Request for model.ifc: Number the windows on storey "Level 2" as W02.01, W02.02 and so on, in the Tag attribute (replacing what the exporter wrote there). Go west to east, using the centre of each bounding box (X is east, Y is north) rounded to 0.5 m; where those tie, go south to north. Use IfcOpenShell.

First a look at what the model holds.

```python
import ifcopenshell
import ifcopenshell.util.element
import ifcopenshell.util.placement

model = ifcopenshell.open("model.ifc")
print(model.schema)
storey = next(s for s in model.by_type("IfcBuildingStorey") if s.Name == "Level 2")
windows = [e for e in ifcopenshell.util.element.get_decomposition(storey) if e.is_a("IfcWindow")]
for e in sorted(windows, key=lambda e: e.id()):
    origin = ifcopenshell.util.placement.get_local_placement(e.ObjectPlacement)[:3, 3]
    print(e.id(), e.Tag, e.Name, origin.round(2) + 0.0, sep=" | ")
```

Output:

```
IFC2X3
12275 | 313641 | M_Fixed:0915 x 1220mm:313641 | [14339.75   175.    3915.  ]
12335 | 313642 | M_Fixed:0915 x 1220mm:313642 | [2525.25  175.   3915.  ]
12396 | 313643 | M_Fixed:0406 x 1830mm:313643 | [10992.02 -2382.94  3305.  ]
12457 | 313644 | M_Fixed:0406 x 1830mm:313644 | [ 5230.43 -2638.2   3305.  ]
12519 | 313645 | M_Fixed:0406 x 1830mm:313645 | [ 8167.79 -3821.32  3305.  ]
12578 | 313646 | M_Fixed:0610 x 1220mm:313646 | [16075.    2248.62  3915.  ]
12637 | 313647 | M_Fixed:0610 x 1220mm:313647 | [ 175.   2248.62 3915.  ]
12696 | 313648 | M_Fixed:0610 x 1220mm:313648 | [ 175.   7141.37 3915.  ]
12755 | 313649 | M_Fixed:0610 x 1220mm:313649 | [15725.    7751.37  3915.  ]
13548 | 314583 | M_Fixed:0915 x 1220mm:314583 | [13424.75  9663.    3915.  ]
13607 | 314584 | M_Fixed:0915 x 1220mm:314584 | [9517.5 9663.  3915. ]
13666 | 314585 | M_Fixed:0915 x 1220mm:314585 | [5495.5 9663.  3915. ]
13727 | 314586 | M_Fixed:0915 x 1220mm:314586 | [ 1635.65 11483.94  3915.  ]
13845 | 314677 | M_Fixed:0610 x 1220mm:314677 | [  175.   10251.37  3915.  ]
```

```python
import ifcopenshell
import ifcopenshell.geom
import ifcopenshell.util.element
import ifcopenshell.util.shape

model = ifcopenshell.open("model.ifc")
settings = ifcopenshell.geom.settings()
settings.set("use-world-coords", True)


def centre(element):
    shape = ifcopenshell.geom.create_shape(settings, element)
    return ifcopenshell.util.shape.get_bbox_centroid(shape.geometry)


storey = next(s for s in model.by_type("IfcBuildingStorey") if s.Name == "Level 2")
windows = [e for e in ifcopenshell.util.element.get_decomposition(storey) if e.is_a("IfcWindow")]

# Insertion points can sit at a corner or the storey origin, so sort by the geometry (in metres).
centres = {e: centre(e) for e in windows}
windows.sort(key=lambda e: (round(centres[e][0] / 0.5), centres[e][1]))

for i, e in enumerate(windows, start=1):
    number = f"W02.{i:02d}"
    e.Tag = number
    print(e.id(), number)

model.write("model_v2.ifc")
```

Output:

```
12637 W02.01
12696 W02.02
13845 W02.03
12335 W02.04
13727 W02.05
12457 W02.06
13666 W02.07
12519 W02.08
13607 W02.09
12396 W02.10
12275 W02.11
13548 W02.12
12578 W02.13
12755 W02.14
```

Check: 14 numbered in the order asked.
